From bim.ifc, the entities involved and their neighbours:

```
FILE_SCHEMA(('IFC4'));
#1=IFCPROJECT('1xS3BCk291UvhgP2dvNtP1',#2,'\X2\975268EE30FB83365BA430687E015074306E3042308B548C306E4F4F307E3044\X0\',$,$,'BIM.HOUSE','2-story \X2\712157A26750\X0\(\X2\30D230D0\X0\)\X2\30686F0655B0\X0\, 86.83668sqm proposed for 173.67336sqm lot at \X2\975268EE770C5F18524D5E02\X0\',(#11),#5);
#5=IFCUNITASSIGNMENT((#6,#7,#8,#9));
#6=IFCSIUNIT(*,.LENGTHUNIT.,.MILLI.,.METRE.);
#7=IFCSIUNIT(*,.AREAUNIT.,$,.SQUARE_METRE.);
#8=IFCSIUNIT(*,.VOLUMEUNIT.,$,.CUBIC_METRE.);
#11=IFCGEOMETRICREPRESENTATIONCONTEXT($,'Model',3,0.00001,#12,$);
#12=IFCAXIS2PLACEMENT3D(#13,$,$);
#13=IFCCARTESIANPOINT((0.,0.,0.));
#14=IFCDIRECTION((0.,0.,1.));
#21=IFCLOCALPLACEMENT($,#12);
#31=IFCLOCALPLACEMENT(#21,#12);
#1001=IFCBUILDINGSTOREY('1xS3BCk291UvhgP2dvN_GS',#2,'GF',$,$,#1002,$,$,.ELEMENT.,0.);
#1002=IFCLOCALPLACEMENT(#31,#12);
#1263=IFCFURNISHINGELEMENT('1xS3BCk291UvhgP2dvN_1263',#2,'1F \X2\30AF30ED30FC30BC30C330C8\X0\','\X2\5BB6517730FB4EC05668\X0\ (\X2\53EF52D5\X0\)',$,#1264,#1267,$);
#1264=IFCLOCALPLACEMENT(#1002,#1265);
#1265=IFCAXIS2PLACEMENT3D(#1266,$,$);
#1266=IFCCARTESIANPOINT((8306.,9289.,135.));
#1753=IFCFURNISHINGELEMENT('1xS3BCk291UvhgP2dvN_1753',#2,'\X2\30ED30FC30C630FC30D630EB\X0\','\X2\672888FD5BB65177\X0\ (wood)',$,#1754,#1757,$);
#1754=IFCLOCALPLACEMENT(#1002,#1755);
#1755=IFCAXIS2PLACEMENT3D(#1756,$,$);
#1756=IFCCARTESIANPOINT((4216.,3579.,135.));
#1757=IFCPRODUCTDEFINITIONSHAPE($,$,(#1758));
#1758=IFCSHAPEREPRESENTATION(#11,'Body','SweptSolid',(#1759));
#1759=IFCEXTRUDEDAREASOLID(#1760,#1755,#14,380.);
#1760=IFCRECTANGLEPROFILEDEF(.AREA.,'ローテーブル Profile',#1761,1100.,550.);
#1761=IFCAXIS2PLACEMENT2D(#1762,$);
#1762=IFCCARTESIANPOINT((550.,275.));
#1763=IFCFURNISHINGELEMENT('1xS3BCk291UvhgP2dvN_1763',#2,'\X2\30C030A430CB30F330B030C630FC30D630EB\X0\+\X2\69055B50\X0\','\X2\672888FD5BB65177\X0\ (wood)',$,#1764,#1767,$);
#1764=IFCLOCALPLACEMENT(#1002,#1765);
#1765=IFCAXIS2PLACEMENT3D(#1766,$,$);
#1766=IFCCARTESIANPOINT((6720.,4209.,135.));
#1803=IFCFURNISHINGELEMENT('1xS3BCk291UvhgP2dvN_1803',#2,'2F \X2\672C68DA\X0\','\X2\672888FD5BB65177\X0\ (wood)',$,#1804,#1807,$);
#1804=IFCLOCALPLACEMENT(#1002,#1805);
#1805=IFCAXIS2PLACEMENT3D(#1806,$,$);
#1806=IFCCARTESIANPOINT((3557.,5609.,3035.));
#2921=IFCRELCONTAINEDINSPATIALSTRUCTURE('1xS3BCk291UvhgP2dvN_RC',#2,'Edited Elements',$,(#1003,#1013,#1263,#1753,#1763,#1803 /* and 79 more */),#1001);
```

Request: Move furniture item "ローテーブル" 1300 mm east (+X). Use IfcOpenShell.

```python
import ifcopenshell
import ifcopenshell.api.geometry
import ifcopenshell.util.placement

model = ifcopenshell.open("bim.ifc")

item = model.by_id(1753)
matrix = ifcopenshell.util.placement.get_local_placement(item.ObjectPlacement)
matrix[0, 3] += 1300.0
ifcopenshell.api.geometry.edit_object_placement(model, product=item, matrix=matrix, is_si=False)

print(ifcopenshell.util.placement.get_local_placement(item.ObjectPlacement).round(3) + 0.0)

model.write("bim_rev.ifc")
```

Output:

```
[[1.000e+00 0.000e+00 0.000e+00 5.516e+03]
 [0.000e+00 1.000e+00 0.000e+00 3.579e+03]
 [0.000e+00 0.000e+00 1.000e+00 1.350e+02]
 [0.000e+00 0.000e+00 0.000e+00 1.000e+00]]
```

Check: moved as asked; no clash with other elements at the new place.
